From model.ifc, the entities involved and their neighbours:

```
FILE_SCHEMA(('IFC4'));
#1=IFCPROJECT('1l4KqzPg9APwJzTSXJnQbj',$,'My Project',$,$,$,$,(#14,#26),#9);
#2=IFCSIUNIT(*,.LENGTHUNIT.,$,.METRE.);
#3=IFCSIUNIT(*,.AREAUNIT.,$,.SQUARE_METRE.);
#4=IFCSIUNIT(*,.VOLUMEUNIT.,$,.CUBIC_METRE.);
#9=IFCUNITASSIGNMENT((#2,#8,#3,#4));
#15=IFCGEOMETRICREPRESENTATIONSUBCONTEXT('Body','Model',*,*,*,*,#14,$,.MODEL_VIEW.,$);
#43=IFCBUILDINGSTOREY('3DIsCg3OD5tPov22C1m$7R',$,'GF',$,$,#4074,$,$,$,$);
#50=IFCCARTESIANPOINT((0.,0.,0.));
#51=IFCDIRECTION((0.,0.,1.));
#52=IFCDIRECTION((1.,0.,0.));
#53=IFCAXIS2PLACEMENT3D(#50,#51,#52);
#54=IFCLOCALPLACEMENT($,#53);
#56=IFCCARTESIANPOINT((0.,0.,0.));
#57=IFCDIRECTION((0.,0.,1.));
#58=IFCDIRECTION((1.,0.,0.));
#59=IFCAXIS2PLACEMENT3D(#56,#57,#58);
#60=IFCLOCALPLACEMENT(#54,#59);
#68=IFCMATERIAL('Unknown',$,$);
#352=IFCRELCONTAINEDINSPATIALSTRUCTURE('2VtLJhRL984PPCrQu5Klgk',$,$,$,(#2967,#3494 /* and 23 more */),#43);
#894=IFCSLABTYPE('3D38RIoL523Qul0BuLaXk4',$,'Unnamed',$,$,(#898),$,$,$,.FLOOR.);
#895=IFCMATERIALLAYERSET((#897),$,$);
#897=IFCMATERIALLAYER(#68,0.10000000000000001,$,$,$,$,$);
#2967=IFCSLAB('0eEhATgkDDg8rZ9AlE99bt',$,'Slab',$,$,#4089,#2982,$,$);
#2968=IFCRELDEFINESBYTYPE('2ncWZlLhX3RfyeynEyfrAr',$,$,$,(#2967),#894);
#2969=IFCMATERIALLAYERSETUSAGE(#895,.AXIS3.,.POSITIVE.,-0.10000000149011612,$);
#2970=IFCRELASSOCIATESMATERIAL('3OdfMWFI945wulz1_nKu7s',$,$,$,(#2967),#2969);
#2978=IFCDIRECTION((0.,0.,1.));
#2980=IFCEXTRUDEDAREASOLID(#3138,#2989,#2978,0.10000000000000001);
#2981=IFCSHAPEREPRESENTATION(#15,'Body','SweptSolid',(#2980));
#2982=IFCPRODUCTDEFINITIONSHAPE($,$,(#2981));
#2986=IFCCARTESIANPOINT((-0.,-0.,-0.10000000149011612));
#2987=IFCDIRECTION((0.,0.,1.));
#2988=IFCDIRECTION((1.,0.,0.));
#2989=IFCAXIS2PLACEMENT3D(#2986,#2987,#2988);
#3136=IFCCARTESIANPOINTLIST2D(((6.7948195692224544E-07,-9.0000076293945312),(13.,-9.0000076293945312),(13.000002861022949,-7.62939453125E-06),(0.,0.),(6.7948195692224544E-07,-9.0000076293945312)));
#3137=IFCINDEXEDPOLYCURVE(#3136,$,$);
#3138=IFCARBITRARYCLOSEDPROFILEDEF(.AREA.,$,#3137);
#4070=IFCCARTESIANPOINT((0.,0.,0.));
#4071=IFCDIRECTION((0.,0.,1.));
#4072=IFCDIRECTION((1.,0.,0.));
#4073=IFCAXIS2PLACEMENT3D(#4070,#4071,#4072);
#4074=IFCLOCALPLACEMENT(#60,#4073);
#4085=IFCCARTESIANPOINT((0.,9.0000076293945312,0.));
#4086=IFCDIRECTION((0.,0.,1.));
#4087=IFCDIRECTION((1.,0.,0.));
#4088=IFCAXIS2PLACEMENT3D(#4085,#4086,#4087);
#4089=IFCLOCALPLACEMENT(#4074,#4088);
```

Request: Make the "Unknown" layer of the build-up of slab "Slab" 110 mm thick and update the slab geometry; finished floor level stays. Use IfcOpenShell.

```python
import ifcopenshell
import ifcopenshell.util.element
import ifcopenshell.util.representation
import ifcopenshell.util.unit

model = ifcopenshell.open("model.ifc")
unit_scale = ifcopenshell.util.unit.calculate_unit_scale(model)

layer_set = model.by_id(895)
layer = next(l for l in layer_set.MaterialLayers if l.Material and l.Material.Name == "Unknown")
change = 0.11 / unit_scale - layer.LayerThickness
layer.LayerThickness += change

# Geometry does not follow the layer set by itself.
slabs = [e for e in ifcopenshell.util.element.get_elements_by_material(model, layer_set) if e.is_a("IfcSlab")]
for slab in sorted(slabs, key=lambda e: e.id()):
    body = ifcopenshell.util.representation.get_representation(slab, "Model", "Body")
    solid = body.Items[0]
    old_depth = solid.Depth
    solid.Depth += change
    # Extruded upwards: lower the start of the extrusion so the top stays.
    x, y, z = solid.Position.Location.Coordinates
    solid.Position.Location = model.createIfcCartesianPoint((x, y, z - change))
    print(slab.id(), f"{old_depth:g} -> {solid.Depth:g}")

# The layers are counted up from the underside, which has moved.
for usage in {ifcopenshell.util.element.get_material(slab) for slab in slabs}:
    usage.OffsetFromReferenceLine -= change

model.write("model_v2.ifc")
```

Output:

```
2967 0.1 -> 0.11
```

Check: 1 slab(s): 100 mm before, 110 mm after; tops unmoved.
